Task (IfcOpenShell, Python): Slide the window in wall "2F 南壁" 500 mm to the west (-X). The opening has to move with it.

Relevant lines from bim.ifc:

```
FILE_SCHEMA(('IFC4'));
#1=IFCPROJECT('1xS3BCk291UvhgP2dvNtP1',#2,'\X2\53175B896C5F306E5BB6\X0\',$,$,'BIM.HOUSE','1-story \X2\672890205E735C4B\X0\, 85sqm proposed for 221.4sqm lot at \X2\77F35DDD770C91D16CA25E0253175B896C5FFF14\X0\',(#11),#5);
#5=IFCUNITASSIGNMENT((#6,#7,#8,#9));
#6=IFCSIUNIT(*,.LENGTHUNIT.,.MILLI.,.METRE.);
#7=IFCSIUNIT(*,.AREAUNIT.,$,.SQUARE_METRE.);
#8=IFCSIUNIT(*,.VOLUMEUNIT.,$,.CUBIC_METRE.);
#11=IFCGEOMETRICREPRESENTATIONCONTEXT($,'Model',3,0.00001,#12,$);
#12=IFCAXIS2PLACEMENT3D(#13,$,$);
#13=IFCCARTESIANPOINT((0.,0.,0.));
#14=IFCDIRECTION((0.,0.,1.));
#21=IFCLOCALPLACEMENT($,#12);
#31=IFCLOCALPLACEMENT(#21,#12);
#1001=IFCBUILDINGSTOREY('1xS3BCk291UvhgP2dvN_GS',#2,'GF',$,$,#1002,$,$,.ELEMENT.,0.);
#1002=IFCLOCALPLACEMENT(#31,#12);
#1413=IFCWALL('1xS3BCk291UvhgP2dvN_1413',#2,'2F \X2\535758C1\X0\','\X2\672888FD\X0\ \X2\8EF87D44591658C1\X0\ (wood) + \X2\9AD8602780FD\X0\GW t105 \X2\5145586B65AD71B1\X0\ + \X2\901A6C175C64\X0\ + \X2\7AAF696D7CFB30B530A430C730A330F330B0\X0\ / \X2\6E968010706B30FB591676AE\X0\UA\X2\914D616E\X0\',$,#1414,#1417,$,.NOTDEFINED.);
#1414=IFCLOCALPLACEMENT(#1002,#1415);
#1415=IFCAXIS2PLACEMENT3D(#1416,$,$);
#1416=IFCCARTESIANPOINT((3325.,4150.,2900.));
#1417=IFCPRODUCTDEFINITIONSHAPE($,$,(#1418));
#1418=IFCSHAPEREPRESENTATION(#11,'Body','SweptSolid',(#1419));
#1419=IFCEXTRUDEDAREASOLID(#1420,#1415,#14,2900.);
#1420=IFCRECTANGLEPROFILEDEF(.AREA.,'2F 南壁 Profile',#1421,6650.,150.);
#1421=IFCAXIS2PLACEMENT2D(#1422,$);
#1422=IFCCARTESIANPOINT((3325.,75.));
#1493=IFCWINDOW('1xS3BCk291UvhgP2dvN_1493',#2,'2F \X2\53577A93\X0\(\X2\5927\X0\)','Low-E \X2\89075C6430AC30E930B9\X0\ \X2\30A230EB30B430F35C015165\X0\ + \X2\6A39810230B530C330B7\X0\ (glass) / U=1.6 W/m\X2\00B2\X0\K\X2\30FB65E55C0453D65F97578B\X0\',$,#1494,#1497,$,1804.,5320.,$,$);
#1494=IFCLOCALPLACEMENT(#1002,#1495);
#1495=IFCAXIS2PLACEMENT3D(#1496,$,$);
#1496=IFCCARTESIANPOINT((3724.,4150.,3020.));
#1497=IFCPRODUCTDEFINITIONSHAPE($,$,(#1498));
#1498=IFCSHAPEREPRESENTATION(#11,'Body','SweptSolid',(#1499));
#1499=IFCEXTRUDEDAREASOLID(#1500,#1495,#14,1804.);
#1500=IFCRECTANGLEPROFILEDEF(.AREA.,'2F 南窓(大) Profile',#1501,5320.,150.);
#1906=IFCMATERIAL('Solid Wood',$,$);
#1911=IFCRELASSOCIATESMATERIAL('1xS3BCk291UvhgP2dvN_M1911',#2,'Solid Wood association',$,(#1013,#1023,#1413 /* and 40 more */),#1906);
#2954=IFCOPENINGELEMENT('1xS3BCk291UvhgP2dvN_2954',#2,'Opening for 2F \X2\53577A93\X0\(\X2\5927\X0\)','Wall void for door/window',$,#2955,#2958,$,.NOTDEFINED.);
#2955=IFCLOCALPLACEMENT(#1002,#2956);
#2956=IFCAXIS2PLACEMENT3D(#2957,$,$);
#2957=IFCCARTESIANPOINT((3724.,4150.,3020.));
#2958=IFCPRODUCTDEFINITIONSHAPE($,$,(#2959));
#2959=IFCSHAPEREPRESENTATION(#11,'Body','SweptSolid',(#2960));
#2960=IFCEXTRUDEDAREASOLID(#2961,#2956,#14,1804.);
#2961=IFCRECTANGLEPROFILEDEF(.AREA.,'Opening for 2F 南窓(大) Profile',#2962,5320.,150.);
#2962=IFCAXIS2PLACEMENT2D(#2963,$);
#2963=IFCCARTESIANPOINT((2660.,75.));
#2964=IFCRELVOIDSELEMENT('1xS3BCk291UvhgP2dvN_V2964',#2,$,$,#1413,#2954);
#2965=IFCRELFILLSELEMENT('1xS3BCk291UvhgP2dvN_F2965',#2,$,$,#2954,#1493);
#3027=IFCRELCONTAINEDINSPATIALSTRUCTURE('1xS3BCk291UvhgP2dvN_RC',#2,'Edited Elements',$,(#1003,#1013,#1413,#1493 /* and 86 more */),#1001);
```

```python
import ifcopenshell
import ifcopenshell.api.geometry
import ifcopenshell.util.placement
import ifcopenshell.util.unit

model = ifcopenshell.open("bim.ifc")
unit_scale = ifcopenshell.util.unit.calculate_unit_scale(model)

window = model.by_id(1493)
opening = window.FillsVoids[0].RelatingOpeningElement
wall = opening.VoidsElements[0].RelatingBuildingElement

wall_matrix = ifcopenshell.util.placement.get_local_placement(wall.ObjectPlacement)
shift = wall_matrix[:3, 0] * -0.5 / unit_scale
before = ifcopenshell.util.placement.get_local_placement(window.ObjectPlacement)[:3, 3].copy()

# The window is not placed relative to its opening, so move both.
for product in (opening, window):
    matrix = ifcopenshell.util.placement.get_local_placement(product.ObjectPlacement)
    matrix[:3, 3] += shift
    ifcopenshell.api.geometry.edit_object_placement(model, product=product, matrix=matrix, is_si=False)

after = ifcopenshell.util.placement.get_local_placement(window.ObjectPlacement)[:3, 3]
print("window moved by", (after - before).round(3) + 0.0)

model.write("bim_edited.ifc")
```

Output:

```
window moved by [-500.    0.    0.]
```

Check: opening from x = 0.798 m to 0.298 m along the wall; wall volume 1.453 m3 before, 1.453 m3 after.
